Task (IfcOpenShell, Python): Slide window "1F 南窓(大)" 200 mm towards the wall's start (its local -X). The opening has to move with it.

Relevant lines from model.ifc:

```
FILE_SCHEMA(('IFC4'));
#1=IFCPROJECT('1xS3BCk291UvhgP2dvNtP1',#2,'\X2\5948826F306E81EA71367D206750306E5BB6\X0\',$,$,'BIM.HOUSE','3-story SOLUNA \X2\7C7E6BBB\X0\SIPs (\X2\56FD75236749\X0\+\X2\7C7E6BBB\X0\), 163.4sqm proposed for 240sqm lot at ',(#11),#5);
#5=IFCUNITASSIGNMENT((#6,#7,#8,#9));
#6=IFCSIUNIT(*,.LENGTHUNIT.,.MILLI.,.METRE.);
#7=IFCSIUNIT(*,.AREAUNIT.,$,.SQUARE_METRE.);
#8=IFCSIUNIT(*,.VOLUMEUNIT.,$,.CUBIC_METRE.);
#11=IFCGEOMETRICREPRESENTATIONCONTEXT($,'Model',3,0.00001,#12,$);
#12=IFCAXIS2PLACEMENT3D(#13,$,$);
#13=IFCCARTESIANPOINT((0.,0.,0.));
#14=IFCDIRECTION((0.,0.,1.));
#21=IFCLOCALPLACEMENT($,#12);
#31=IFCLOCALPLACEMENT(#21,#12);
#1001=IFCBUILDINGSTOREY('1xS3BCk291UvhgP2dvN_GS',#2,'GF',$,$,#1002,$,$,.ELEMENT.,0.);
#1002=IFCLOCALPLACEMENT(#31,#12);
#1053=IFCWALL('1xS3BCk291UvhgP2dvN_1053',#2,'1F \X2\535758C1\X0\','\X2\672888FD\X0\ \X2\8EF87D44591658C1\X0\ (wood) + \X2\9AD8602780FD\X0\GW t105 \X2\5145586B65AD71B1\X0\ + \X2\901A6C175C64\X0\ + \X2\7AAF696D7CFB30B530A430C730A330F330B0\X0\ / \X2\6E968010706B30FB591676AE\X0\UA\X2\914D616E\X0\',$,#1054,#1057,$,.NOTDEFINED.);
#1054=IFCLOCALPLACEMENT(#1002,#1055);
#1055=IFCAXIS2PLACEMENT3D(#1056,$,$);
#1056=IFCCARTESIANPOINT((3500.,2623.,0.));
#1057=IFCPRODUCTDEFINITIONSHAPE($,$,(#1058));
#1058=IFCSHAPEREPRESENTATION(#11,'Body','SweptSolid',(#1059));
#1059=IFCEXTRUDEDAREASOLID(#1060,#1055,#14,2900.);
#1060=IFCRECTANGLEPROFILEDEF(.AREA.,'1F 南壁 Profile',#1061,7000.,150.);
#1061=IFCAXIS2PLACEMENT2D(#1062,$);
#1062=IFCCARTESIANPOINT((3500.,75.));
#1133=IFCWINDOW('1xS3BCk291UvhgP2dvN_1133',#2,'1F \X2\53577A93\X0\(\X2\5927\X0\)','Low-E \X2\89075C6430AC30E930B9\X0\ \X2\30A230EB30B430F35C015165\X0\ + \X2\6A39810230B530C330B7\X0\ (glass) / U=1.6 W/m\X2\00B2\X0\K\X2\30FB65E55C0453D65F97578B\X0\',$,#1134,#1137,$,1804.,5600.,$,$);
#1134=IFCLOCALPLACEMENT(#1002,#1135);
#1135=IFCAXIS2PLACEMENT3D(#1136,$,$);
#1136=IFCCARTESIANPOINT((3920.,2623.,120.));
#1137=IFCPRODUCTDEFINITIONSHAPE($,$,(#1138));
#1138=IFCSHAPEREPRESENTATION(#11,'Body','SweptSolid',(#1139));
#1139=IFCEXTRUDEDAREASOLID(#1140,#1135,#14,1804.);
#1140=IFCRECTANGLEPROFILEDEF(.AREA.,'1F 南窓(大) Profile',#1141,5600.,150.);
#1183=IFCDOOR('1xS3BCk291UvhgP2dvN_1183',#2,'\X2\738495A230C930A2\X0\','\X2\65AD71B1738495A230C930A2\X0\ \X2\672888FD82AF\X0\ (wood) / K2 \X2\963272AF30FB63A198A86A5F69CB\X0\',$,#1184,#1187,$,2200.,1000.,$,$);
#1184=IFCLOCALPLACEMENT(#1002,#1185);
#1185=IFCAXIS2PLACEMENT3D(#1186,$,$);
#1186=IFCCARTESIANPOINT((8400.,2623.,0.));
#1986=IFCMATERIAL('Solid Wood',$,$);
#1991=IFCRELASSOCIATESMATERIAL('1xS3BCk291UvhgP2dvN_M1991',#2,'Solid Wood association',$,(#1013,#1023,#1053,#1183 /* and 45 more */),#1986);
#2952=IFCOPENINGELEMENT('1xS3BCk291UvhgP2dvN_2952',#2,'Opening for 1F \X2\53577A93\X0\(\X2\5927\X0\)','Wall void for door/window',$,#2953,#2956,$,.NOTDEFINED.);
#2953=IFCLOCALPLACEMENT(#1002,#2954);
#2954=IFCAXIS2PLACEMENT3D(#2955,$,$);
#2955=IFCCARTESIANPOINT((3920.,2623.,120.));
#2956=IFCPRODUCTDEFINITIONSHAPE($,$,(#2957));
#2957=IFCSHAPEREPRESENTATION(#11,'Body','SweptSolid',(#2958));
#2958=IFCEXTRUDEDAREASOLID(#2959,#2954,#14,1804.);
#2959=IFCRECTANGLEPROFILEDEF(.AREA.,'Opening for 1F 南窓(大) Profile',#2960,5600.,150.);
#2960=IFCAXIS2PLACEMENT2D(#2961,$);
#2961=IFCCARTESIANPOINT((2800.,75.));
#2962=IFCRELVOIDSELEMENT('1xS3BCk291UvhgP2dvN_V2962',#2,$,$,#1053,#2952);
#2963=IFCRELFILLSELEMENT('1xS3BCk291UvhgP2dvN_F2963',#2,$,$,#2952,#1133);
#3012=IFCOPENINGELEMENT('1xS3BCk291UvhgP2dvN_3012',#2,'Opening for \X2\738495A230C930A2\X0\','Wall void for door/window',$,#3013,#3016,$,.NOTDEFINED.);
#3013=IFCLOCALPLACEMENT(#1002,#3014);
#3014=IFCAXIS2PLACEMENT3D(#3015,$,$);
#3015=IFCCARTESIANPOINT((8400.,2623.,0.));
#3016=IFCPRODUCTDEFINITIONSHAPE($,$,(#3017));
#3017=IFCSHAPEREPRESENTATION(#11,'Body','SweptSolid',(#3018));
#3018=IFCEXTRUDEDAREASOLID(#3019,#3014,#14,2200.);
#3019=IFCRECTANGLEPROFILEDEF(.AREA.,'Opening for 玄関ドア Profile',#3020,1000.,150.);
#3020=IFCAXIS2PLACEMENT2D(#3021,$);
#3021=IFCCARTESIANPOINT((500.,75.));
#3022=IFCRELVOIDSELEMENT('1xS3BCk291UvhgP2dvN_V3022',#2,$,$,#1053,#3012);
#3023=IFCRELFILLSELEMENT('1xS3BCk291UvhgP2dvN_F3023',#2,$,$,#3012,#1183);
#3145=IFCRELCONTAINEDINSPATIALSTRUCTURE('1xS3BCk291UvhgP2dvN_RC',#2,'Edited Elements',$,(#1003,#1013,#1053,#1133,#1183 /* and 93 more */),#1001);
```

```python
import ifcopenshell
import ifcopenshell.api.geometry
import ifcopenshell.util.placement
import ifcopenshell.util.unit

model = ifcopenshell.open("model.ifc")
unit_scale = ifcopenshell.util.unit.calculate_unit_scale(model)

window = model.by_id(1133)
opening = window.FillsVoids[0].RelatingOpeningElement
wall = opening.VoidsElements[0].RelatingBuildingElement

wall_matrix = ifcopenshell.util.placement.get_local_placement(wall.ObjectPlacement)
shift = wall_matrix[:3, 0] * -0.2 / unit_scale
before = ifcopenshell.util.placement.get_local_placement(window.ObjectPlacement)[:3, 3].copy()

# The window is not placed relative to its opening, so move both.
for product in (opening, window):
    matrix = ifcopenshell.util.placement.get_local_placement(product.ObjectPlacement)
    matrix[:3, 3] += shift
    ifcopenshell.api.geometry.edit_object_placement(model, product=product, matrix=matrix, is_si=False)

after = ifcopenshell.util.placement.get_local_placement(window.ObjectPlacement)[:3, 3]
print("window moved by", (after - before).round(3) + 0.0)

model.write("model_edited.ifc")
```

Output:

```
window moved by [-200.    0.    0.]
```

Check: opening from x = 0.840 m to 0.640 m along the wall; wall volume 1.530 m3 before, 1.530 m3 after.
